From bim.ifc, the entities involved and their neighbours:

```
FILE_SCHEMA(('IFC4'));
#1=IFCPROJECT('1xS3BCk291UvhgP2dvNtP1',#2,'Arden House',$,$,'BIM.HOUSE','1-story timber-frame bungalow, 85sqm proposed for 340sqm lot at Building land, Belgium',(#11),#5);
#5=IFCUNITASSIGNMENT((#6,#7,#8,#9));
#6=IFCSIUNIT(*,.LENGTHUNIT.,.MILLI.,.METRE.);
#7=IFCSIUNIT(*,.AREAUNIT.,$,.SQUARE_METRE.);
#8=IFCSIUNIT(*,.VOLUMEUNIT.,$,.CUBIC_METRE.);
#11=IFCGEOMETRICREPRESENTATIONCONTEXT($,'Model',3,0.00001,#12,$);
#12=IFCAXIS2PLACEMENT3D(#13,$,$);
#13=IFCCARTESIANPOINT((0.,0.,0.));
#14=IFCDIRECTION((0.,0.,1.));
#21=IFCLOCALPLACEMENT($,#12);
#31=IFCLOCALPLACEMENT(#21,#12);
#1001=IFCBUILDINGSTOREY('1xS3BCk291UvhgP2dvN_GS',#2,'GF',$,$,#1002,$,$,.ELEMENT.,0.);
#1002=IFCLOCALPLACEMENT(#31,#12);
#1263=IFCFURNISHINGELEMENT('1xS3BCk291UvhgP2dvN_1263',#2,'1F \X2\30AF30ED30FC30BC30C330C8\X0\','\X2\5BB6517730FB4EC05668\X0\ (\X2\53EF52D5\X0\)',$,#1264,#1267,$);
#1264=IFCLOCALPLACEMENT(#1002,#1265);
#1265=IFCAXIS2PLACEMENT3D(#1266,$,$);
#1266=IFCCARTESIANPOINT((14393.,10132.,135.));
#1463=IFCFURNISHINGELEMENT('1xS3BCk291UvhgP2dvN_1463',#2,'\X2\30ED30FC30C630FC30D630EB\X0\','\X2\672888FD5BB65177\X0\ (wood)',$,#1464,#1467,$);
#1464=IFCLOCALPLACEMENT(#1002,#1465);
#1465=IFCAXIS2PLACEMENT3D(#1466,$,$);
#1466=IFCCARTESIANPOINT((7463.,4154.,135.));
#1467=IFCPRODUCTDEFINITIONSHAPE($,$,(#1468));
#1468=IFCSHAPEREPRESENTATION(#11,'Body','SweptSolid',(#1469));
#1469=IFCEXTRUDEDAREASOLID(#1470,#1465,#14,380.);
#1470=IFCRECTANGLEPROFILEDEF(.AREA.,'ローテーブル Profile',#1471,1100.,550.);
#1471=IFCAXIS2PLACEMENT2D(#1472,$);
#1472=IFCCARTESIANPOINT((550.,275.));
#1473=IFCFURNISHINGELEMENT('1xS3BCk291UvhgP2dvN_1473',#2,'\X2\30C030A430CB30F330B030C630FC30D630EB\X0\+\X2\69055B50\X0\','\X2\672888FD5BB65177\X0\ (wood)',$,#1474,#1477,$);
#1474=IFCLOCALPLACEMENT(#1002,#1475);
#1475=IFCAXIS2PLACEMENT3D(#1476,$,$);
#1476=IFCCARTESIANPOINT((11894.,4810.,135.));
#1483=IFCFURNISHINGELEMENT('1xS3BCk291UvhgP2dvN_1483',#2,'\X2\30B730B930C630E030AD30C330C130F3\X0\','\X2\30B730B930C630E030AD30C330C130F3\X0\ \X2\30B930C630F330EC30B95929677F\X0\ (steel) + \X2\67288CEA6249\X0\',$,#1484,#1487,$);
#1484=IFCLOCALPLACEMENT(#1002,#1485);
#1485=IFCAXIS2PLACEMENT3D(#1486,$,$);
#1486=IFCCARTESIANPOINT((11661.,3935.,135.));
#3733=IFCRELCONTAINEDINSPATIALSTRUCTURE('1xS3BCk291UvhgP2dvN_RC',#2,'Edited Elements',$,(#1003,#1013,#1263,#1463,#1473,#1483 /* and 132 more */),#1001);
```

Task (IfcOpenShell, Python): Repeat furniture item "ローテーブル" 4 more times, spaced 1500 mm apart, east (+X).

```python
import numpy as np
import ifcopenshell
import ifcopenshell.api.geometry
import ifcopenshell.api.root
import ifcopenshell.util.element
import ifcopenshell.util.placement
import ifcopenshell.util.unit

model = ifcopenshell.open("bim.ifc")
unit_scale = ifcopenshell.util.unit.calculate_unit_scale(model)


def reuse_history(source, copy):
    """copy_class also copies each property set's owner history, people and application; keep the originals."""
    for rel in copy.IsDefinedBy:
        if rel.is_a("IfcRelDefinesByProperties") and (history := rel.RelatingPropertyDefinition.OwnerHistory):
            rel.RelatingPropertyDefinition.OwnerHistory = source.OwnerHistory
            ifcopenshell.util.element.remove_deep2(model, history)


source = model.by_guid("1xS3BCk291UvhgP2dvN_1463")
base = ifcopenshell.util.placement.get_local_placement(source.ObjectPlacement)
step = np.array([1.0, 0.0, 0.0]) * 1.5 / unit_scale

for i in range(1, 5):
    copy = ifcopenshell.api.root.copy_class(model, product=source)
    copy.Representation = ifcopenshell.util.element.copy_deep(
        model, source.Representation, exclude=["IfcGeometricRepresentationContext", "IfcRepresentationMap"]
    )
    reuse_history(source, copy)
    matrix = base.copy()
    matrix[:3, 3] += i * step
    print("added at", matrix[:3, 3].round(3) + 0.0)
    ifcopenshell.api.geometry.edit_object_placement(model, product=copy, matrix=matrix, is_si=False)

model.write("bim_edited.ifc")
```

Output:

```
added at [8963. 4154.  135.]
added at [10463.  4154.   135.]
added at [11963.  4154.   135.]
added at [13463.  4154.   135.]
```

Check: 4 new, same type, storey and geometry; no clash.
